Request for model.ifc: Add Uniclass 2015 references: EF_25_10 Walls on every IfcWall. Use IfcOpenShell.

First a look at what the model holds.

```python
import ifcopenshell

model = ifcopenshell.open("model.ifc")
print(model.schema)
print("classifications:", [c.Name for c in model.by_type("IfcClassification")])
for ifc_class in ("IfcDoor", "IfcRoof", "IfcStair", "IfcWall", "IfcWindow"):
    print(ifc_class, len(model.by_type(ifc_class)))
```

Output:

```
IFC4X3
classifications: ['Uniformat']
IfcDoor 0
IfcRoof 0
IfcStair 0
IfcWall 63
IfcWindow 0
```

```python
import ifcopenshell
import ifcopenshell.api.classification

model = ifcopenshell.open("model.ifc")

system = ifcopenshell.api.classification.add_classification(model, classification="Uniclass 2015")

codes = {
    "IfcWall": ("EF_25_10", "Walls"),
}
for ifc_class, (code, name) in codes.items():
    products = model.by_type(ifc_class)
    ifcopenshell.api.classification.add_reference(
        model, products=products, classification=system, identification=code, name=name
    )
    print(code, len(products))

model.write("model-out.ifc")
```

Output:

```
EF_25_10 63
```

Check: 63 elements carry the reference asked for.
